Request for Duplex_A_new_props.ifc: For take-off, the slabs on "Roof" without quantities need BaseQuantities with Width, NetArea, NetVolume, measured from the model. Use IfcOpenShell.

First a look at what the model holds.

```python
import ifcopenshell
import ifcopenshell.util.element
import ifcopenshell.util.unit

model = ifcopenshell.open("Duplex_A_new_props.ifc")
print(model.schema)
for unit_type in ("LENGTHUNIT", "AREAUNIT", "VOLUMEUNIT"):
    print(unit_type, ifcopenshell.util.unit.calculate_unit_scale(model, unit_type))
storey = next(s for s in model.by_type("IfcBuildingStorey") if s.Name == "Roof")
slabs = [e for e in ifcopenshell.util.element.get_decomposition(storey) if e.is_a("IfcSlab")]
for e in sorted(slabs, key=lambda e: e.id()):
    print(e.id(), e.is_a(), e.Name, list(ifcopenshell.util.element.get_psets(e, qtos_only=True)), sep=" | ")
```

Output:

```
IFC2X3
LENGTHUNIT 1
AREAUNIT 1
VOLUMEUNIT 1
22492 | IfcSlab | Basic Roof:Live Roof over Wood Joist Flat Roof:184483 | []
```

```python
import ifcopenshell
import ifcopenshell.api.pset
import ifcopenshell.geom
import ifcopenshell.util.element
import ifcopenshell.util.shape
import ifcopenshell.util.unit

model = ifcopenshell.open("Duplex_A_new_props.ifc")
unit_scale = ifcopenshell.util.unit.calculate_unit_scale(model)
area_scale = ifcopenshell.util.unit.calculate_unit_scale(model, "AREAUNIT")
volume_scale = ifcopenshell.util.unit.calculate_unit_scale(model, "VOLUMEUNIT")
settings = ifcopenshell.geom.settings()

storey = next(s for s in model.by_type("IfcBuildingStorey") if s.Name == "Roof")
slabs = [e for e in ifcopenshell.util.element.get_decomposition(storey) if e.is_a("IfcSlab")]

for e in sorted(slabs, key=lambda e: e.id()):
    if ifcopenshell.util.element.get_psets(e, qtos_only=True, should_inherit=False):
        continue
    # Geometry comes back in metres, in the element's own axes.
    shape = ifcopenshell.geom.create_shape(settings, e)
    values = {
        "Width": ifcopenshell.util.shape.get_z(shape.geometry) / unit_scale,
        "NetArea": ifcopenshell.util.shape.get_footprint_area(shape.geometry) / area_scale,
        "NetVolume": ifcopenshell.util.shape.get_volume(shape.geometry) / volume_scale,
    }
    qto = ifcopenshell.api.pset.add_qto(model, product=e, name="BaseQuantities")
    ifcopenshell.api.pset.edit_qto(model, qto=qto, properties=values)
    print(e.id(), {k: round(v, 3) for k, v in values.items()})

model.write("Duplex_A_new_props_updated.ifc")
```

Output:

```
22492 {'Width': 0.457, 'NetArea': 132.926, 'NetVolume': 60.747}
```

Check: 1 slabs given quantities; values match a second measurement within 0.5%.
